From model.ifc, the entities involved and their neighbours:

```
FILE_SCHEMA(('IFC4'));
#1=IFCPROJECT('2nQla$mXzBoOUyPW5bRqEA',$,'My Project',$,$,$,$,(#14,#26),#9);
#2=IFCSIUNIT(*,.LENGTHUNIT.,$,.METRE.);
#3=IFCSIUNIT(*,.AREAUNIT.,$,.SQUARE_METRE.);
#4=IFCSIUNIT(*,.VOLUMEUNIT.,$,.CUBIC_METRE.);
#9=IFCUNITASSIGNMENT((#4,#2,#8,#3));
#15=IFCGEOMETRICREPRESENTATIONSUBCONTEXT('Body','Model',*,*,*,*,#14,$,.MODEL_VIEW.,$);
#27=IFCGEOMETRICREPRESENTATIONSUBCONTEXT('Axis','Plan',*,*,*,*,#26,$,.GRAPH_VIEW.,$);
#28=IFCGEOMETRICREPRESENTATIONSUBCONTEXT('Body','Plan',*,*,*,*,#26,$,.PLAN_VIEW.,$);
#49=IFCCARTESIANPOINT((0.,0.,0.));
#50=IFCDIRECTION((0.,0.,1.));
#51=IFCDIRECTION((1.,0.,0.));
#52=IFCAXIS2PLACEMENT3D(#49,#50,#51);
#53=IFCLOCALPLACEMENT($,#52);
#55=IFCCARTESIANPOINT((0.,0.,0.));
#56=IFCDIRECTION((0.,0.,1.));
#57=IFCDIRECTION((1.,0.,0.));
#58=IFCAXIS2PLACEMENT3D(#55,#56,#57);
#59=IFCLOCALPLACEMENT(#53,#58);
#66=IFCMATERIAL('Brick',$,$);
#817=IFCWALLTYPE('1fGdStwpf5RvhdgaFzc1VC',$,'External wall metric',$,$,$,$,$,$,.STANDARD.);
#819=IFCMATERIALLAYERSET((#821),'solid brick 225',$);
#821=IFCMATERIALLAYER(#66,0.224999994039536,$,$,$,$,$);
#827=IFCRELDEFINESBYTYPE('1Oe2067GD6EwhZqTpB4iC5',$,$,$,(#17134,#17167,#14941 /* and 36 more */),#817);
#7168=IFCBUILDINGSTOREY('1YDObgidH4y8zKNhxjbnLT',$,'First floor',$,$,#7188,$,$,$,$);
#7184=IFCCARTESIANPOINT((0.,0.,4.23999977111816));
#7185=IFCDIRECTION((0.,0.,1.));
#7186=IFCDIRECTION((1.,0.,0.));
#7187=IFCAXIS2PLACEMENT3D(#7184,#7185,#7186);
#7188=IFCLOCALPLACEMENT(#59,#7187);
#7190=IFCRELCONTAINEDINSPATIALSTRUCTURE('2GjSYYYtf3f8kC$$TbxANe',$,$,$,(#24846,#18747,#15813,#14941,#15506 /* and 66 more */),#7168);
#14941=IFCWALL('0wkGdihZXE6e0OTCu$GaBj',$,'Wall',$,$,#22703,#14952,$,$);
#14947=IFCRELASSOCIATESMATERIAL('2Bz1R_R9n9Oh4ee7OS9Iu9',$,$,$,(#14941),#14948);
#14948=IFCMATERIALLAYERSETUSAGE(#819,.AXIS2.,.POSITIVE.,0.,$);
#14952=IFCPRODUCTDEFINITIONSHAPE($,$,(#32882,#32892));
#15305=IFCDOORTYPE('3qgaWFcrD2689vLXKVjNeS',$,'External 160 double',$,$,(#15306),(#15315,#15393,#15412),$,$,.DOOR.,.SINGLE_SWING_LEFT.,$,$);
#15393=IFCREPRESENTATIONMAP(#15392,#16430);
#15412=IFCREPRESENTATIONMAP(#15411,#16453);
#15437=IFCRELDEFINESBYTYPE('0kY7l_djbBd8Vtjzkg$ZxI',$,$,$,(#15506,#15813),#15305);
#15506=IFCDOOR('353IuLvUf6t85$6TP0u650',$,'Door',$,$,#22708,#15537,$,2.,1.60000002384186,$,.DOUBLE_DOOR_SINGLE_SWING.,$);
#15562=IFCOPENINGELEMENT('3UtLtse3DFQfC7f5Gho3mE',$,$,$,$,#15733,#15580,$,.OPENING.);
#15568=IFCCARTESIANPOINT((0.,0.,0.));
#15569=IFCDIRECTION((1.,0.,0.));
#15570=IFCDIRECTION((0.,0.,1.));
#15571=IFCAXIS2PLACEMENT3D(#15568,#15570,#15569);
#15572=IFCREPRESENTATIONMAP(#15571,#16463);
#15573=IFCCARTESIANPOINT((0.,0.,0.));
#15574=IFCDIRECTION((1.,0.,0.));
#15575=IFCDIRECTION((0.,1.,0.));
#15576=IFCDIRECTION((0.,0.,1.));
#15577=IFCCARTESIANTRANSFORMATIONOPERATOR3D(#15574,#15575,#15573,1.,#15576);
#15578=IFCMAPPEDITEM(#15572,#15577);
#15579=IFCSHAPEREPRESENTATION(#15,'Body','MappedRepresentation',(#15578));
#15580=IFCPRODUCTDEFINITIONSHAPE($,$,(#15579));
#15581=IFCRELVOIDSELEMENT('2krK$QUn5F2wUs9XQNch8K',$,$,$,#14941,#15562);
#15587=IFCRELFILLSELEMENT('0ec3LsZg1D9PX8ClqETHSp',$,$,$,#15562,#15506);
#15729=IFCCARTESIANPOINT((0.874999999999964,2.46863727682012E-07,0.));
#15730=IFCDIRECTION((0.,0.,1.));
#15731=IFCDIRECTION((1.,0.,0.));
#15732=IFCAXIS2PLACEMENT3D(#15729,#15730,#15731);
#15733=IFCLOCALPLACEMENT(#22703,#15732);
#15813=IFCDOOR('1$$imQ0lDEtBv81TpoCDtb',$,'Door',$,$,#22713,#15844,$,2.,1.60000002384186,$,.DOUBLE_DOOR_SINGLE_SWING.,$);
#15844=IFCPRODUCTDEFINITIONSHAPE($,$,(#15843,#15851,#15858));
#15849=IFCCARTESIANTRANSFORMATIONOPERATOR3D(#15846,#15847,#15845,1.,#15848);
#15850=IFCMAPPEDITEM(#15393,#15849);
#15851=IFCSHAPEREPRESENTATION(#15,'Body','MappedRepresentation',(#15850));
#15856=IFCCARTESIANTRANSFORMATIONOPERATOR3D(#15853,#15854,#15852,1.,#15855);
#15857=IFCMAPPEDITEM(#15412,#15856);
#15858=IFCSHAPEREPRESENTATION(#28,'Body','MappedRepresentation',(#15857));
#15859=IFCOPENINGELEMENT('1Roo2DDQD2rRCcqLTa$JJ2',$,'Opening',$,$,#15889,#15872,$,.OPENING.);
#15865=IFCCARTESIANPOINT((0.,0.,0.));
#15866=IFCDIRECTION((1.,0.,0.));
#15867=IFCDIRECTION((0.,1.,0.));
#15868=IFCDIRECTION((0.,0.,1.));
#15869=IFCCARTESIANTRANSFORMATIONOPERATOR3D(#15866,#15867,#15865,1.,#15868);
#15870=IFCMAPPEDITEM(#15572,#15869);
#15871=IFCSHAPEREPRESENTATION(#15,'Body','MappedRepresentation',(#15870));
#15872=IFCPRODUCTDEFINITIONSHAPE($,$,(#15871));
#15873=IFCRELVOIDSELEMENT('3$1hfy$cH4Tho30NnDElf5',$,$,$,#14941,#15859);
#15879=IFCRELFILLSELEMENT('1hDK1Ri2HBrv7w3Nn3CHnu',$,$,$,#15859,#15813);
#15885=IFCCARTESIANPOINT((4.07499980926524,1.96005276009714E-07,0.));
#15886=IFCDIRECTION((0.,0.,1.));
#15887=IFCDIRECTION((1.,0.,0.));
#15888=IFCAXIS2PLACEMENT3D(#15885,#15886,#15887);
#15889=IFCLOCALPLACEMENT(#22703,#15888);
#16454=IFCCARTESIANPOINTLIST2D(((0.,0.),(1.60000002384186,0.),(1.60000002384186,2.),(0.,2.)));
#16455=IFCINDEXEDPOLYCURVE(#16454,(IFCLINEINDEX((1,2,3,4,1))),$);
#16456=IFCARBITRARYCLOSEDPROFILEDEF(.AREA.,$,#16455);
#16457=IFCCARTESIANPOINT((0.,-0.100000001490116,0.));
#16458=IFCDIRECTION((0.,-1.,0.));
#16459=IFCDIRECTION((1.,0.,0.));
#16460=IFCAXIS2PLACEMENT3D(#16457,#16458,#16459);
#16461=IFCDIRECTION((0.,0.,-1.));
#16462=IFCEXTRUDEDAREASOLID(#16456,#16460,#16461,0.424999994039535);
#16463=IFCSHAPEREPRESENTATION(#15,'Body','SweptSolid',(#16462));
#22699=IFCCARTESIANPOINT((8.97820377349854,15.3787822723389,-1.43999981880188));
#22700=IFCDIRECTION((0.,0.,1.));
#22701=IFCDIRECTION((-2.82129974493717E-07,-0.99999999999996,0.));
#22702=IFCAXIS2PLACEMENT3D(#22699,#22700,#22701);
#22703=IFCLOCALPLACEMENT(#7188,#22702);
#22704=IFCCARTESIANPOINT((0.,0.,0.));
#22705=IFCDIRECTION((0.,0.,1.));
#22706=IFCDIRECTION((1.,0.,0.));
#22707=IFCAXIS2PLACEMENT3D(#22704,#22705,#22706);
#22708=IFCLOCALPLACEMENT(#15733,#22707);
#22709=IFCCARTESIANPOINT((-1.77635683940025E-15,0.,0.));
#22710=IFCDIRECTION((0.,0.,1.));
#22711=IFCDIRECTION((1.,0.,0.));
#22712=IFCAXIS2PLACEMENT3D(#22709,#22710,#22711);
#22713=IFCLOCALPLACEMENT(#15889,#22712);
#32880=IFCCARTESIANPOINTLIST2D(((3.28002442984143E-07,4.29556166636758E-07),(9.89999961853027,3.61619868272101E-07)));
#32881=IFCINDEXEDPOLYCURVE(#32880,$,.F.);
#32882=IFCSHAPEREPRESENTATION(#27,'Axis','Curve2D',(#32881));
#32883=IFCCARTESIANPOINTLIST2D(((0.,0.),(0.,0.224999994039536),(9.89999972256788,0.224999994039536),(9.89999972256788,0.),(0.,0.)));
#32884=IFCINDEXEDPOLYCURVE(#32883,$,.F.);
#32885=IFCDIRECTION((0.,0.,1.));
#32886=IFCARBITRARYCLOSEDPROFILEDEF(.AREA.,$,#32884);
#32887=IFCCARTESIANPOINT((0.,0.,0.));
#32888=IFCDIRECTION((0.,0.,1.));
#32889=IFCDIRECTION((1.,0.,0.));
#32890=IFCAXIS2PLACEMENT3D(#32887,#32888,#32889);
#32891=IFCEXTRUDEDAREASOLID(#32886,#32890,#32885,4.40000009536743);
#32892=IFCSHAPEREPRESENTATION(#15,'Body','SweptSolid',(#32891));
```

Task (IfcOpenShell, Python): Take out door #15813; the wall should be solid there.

```python
import ifcopenshell
import ifcopenshell.api.feature
import ifcopenshell.api.root
import ifcopenshell.geom
import ifcopenshell.util.shape

model = ifcopenshell.open("model.ifc")
settings = ifcopenshell.geom.settings()


def volume(element):
    """Net volume in cubic metres, openings subtracted."""
    shape = ifcopenshell.geom.create_shape(settings, element)
    return ifcopenshell.util.shape.get_volume(shape.geometry)


door = model.by_guid("1$$imQ0lDEtBv81TpoCDtb")
opening = door.FillsVoids[0].RelatingOpeningElement
wall = opening.VoidsElements[0].RelatingBuildingElement
before = volume(wall)

ifcopenshell.api.root.remove_product(model, product=door)
ifcopenshell.api.feature.remove_feature(model, feature=opening)

after = volume(wall)

print(f"wall volume {before:.3f} -> {after:.3f} m3")

model.write("model_updated.ifc")
```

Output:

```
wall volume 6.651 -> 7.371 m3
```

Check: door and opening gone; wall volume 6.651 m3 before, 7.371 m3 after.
